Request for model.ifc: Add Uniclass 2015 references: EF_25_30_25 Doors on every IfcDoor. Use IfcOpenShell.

First a look at what the model holds.

```python
import ifcopenshell

model = ifcopenshell.open("model.ifc")
print(model.schema)
print("classifications:", [c.Name for c in model.by_type("IfcClassification")])
for ifc_class in ("IfcDoor", "IfcRoof", "IfcStair", "IfcWall", "IfcWindow"):
    print(ifc_class, len(model.by_type(ifc_class)))
```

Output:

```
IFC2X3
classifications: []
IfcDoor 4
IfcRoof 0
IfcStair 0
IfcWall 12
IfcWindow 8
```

```python
import ifcopenshell
import ifcopenshell.api.classification

model = ifcopenshell.open("model.ifc")

# IFC2X3 requires Source and Edition and has no link from the project to the system.
system = model.create_entity("IfcClassification", Source="NBS", Edition="2015", Name="Uniclass 2015")

codes = {
    "IfcDoor": ("EF_25_30_25", "Doors"),
}
for ifc_class, (code, name) in codes.items():
    products = model.by_type(ifc_class)
    ifcopenshell.api.classification.add_reference(
        model, products=products, classification=system, identification=code, name=name
    )
    print(code, len(products))

model.write("model_updated.ifc")
```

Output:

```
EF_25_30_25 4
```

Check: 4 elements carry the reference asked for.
